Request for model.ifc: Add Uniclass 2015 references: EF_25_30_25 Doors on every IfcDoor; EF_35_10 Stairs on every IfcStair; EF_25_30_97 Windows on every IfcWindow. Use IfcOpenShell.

First a look at what the model holds.

```python
import ifcopenshell

model = ifcopenshell.open("model.ifc")
print(model.schema)
print("classifications:", [c.Name for c in model.by_type("IfcClassification")])
for ifc_class in ("IfcDoor", "IfcRoof", "IfcStair", "IfcWall", "IfcWindow"):
    print(ifc_class, len(model.by_type(ifc_class)))
```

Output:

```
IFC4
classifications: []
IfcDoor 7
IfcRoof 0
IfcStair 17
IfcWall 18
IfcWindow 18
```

```python
import ifcopenshell
import ifcopenshell.api.classification

model = ifcopenshell.open("model.ifc")

system = ifcopenshell.api.classification.add_classification(model, classification="Uniclass 2015")

codes = {
    "IfcDoor": ("EF_25_30_25", "Doors"),
    "IfcStair": ("EF_35_10", "Stairs"),
    "IfcWindow": ("EF_25_30_97", "Windows"),
}
for ifc_class, (code, name) in codes.items():
    products = model.by_type(ifc_class)
    ifcopenshell.api.classification.add_reference(
        model, products=products, classification=system, identification=code, name=name
    )
    print(code, len(products))

model.write("model_rev.ifc")
```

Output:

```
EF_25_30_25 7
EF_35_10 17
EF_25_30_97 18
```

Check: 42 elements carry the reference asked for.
